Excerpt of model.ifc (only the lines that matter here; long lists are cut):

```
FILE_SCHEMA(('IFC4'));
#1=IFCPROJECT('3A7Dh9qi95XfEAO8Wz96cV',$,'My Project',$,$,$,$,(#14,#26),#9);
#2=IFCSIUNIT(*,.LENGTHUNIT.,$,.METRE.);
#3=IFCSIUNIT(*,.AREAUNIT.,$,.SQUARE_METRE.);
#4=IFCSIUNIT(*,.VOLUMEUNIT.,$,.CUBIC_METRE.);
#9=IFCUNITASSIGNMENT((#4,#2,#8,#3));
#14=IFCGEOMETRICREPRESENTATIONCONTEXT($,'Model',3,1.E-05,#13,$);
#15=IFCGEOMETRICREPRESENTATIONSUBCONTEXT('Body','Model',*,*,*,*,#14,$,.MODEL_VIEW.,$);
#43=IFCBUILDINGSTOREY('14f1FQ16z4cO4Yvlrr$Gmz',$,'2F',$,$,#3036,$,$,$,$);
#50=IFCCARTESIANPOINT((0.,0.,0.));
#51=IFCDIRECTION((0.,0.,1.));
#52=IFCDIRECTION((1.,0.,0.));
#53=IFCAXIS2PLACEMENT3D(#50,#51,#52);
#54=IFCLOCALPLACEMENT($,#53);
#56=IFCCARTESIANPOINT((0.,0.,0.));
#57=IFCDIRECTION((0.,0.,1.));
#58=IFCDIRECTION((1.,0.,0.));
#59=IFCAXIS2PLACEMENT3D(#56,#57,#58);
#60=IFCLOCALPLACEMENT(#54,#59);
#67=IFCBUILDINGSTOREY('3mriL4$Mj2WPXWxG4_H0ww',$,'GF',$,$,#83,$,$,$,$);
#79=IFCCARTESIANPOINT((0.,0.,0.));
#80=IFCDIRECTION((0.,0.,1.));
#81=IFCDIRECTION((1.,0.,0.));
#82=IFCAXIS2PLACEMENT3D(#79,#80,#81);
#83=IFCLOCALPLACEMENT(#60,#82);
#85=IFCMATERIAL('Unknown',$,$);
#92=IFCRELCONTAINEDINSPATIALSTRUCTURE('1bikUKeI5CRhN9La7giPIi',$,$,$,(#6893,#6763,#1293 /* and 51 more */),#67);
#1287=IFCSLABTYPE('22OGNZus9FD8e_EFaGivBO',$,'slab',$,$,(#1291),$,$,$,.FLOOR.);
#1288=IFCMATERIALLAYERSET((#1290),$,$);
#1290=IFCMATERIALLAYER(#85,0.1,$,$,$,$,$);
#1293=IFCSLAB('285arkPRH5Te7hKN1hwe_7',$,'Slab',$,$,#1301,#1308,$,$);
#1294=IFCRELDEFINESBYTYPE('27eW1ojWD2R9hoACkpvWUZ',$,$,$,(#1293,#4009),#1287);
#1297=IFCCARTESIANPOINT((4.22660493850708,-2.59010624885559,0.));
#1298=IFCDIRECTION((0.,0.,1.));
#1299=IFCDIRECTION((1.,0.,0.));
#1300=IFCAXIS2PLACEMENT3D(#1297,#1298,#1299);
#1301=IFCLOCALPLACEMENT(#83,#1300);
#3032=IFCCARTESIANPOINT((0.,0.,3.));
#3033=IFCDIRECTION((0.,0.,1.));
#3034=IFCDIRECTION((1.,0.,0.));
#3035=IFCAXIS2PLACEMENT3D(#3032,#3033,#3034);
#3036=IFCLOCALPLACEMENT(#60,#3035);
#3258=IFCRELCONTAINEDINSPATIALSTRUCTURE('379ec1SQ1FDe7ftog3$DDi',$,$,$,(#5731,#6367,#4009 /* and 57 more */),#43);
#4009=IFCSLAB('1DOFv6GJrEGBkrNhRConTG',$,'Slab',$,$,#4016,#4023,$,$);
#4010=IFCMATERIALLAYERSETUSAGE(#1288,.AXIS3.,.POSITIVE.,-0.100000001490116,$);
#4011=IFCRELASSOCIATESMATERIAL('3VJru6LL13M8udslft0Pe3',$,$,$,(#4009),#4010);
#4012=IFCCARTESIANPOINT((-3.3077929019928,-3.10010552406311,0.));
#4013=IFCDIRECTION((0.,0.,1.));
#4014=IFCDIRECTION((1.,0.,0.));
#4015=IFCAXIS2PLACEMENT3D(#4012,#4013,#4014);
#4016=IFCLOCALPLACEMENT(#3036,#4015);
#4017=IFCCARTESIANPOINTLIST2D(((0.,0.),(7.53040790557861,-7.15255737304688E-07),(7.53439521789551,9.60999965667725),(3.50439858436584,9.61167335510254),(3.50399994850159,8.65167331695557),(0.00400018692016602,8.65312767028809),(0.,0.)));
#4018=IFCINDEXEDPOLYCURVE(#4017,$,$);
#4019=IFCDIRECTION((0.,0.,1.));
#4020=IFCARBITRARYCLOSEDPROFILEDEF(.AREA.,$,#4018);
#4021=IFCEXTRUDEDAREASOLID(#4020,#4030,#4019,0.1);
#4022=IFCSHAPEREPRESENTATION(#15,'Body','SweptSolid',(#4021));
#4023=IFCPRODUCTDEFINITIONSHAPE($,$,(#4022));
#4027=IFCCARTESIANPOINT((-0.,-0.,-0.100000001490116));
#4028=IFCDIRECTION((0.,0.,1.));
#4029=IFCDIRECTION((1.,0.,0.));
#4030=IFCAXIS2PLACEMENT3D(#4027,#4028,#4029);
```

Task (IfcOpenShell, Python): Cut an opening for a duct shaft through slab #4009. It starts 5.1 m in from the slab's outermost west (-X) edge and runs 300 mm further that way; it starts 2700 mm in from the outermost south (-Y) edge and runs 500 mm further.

```python
import numpy as np
import ifcopenshell
import ifcopenshell.api.feature
import ifcopenshell.api.geometry
import ifcopenshell.api.root
import ifcopenshell.geom
import ifcopenshell.util.placement
import ifcopenshell.util.representation
import ifcopenshell.util.shape
import ifcopenshell.util.unit

model = ifcopenshell.open("model.ifc")
unit_scale = ifcopenshell.util.unit.calculate_unit_scale(model)
settings = ifcopenshell.geom.settings()


def volume(element):
    """Net volume in cubic metres, openings subtracted."""
    shape = ifcopenshell.geom.create_shape(settings, element)
    return ifcopenshell.util.shape.get_volume(shape.geometry)


slab = model.by_guid("1DOFv6GJrEGBkrNhRConTG")
before = volume(slab)

# Extent in the slab's own axes, in metres. The edges named are its -X and -Y sides.
slab_shape = ifcopenshell.geom.create_shape(settings, slab)
vertices = ifcopenshell.util.shape.get_vertices(slab_shape.geometry)
x_min, y_min, bottom = vertices.min(axis=0)
top = vertices[:, 2].max()

opening = ifcopenshell.api.root.create_entity(model, ifc_class="IfcOpeningElement", name="Duct shaft opening", predefined_type="OPENING")
context = ifcopenshell.util.representation.get_context(model, "Model", "Body", "MODEL_VIEW")
width, depth = 0.3, 0.5
outline = [(0.0, 0.0), (width, 0.0), (width, depth), (0.0, depth), (0.0, 0.0)]
# Overshoot both faces by 50 mm so the cut is clean.
shape = ifcopenshell.api.geometry.add_slab_representation(
    model, context=context, depth=top - bottom + 0.1, polyline=outline
)
ifcopenshell.api.geometry.assign_representation(model, product=opening, representation=shape)

matrix = ifcopenshell.util.placement.get_local_placement(slab.ObjectPlacement)
matrix[:, 3] = matrix @ np.append(np.array([x_min + 5.1, y_min + 2.7, bottom - 0.05]) / unit_scale, 1.0)
ifcopenshell.api.geometry.edit_object_placement(model, product=opening, matrix=matrix, is_si=False)
ifcopenshell.api.feature.add_feature(model, feature=opening, element=slab)

after = volume(slab)

print(f"slab volume {before:.3f} -> {after:.3f} m3")

model.write("model-out.ifc")
```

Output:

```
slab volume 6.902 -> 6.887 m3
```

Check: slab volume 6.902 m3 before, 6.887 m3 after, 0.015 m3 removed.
